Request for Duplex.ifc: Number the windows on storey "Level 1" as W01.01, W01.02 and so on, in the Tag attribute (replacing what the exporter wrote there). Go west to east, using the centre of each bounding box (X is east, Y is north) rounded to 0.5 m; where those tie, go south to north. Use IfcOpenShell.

First a look at what the model holds.

```python
import ifcopenshell
import ifcopenshell.util.element
import ifcopenshell.util.placement

model = ifcopenshell.open("Duplex.ifc")
print(model.schema)
storey = next(s for s in model.by_type("IfcBuildingStorey") if s.Name == "Level 1")
windows = [e for e in ifcopenshell.util.element.get_decomposition(storey) if e.is_a("IfcWindow")]
for e in sorted(windows, key=lambda e: e.id()):
    origin = ifcopenshell.util.placement.get_local_placement(e.ObjectPlacement)[:3, 3]
    print(e.id(), e.Tag, e.Name, origin.round(2) + 0.0, sep=" | ")
```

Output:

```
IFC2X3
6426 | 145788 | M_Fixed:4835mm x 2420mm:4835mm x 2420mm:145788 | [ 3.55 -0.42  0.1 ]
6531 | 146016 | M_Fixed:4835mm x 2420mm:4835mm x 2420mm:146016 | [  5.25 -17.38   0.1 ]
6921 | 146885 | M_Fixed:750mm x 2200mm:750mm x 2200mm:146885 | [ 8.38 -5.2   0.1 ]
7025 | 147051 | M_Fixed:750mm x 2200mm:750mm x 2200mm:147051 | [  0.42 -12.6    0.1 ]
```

```python
import ifcopenshell
import ifcopenshell.geom
import ifcopenshell.util.element
import ifcopenshell.util.shape

model = ifcopenshell.open("Duplex.ifc")
settings = ifcopenshell.geom.settings()
settings.set("use-world-coords", True)


def centre(element):
    shape = ifcopenshell.geom.create_shape(settings, element)
    return ifcopenshell.util.shape.get_bbox_centroid(shape.geometry)


storey = next(s for s in model.by_type("IfcBuildingStorey") if s.Name == "Level 1")
windows = [e for e in ifcopenshell.util.element.get_decomposition(storey) if e.is_a("IfcWindow")]

# Insertion points can sit at a corner or the storey origin, so sort by the geometry (in metres).
centres = {e: centre(e) for e in windows}
windows.sort(key=lambda e: (round(centres[e][0] / 0.5), centres[e][1]))

for i, e in enumerate(windows, start=1):
    number = f"W01.{i:02d}"
    e.Tag = number
    print(e.id(), number)

model.write("Duplex_v2.ifc")
```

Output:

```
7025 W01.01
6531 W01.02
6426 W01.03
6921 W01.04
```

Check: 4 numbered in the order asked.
